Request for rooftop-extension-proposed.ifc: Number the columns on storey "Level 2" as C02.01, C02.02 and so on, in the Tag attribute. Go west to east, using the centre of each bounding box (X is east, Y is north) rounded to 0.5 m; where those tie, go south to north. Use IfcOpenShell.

First a look at what the model holds.

```python
import ifcopenshell
import ifcopenshell.util.element
import ifcopenshell.util.placement

model = ifcopenshell.open("rooftop-extension-proposed.ifc")
print(model.schema)
storey = next(s for s in model.by_type("IfcBuildingStorey") if s.Name == "Level 2")
columns = [e for e in ifcopenshell.util.element.get_decomposition(storey) if e.is_a("IfcColumn")]
for e in sorted(columns, key=lambda e: e.id()):
    origin = ifcopenshell.util.placement.get_local_placement(e.ObjectPlacement)[:3, 3]
    print(e.id(), e.Tag, e.Name, origin.round(2) + 0.0, sep=" | ")
```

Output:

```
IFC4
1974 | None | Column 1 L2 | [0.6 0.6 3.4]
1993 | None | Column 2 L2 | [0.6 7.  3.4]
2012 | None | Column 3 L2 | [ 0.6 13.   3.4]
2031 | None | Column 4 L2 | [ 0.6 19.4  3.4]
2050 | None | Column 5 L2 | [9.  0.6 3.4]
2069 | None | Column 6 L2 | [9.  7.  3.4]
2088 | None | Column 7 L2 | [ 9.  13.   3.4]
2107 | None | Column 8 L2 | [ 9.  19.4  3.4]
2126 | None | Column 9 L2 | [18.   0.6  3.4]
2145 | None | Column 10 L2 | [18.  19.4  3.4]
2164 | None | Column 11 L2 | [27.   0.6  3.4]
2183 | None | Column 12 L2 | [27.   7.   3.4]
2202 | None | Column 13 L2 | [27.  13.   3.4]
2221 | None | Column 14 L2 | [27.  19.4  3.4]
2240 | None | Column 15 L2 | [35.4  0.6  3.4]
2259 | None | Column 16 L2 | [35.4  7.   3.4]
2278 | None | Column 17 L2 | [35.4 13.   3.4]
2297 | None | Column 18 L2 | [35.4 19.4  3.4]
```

```python
import ifcopenshell
import ifcopenshell.geom
import ifcopenshell.util.element
import ifcopenshell.util.shape

model = ifcopenshell.open("rooftop-extension-proposed.ifc")
settings = ifcopenshell.geom.settings()
settings.set("use-world-coords", True)


def centre(element):
    shape = ifcopenshell.geom.create_shape(settings, element)
    return ifcopenshell.util.shape.get_bbox_centroid(shape.geometry)


storey = next(s for s in model.by_type("IfcBuildingStorey") if s.Name == "Level 2")
columns = [e for e in ifcopenshell.util.element.get_decomposition(storey) if e.is_a("IfcColumn")]

# Insertion points can sit at a corner or the storey origin, so sort by the geometry (in metres).
centres = {e: centre(e) for e in columns}
columns.sort(key=lambda e: (round(centres[e][0] / 0.5), centres[e][1]))

for i, e in enumerate(columns, start=1):
    number = f"C02.{i:02d}"
    e.Tag = number
    print(e.id(), number)

model.write("rooftop-extension-proposed_edited.ifc")
```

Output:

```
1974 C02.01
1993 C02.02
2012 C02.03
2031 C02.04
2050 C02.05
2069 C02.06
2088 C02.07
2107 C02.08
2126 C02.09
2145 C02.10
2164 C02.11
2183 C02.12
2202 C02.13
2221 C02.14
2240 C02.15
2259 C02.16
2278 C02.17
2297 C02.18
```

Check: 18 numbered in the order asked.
